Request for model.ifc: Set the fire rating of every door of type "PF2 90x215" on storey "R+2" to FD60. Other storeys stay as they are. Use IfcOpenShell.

First a look at what the model holds.

```python
import ifcopenshell
import ifcopenshell.util.element

model = ifcopenshell.open("model.ifc")
print(model.schema)
storey = next(s for s in model.by_type("IfcBuildingStorey") if s.Name == "R+2")
doors = [e for e in ifcopenshell.util.element.get_decomposition(storey) if e.is_a("IfcDoor")]
seen = {}
for e in doors:
    element_type = ifcopenshell.util.element.get_type(e)
    key = (element_type.Name if element_type != e and element_type else None, ifcopenshell.util.element.get_pset(e, "Pset_DoorCommon", "FireRating"))
    seen[key] = seen.get(key, 0) + 1
for (name, value), count in sorted(seen.items(), key=str):
    print(count, "x", name, "|", value)
```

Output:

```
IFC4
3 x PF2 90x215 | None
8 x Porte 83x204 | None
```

```python
import ifcopenshell
import ifcopenshell.api.pset
import ifcopenshell.util.element

model = ifcopenshell.open("model.ifc")

storey = next(s for s in model.by_type("IfcBuildingStorey") if s.Name == "R+2")
doors = [e for e in ifcopenshell.util.element.get_decomposition(storey) if e.is_a("IfcDoor")]

count = 0
for e in doors:
    element_type = ifcopenshell.util.element.get_type(e)
    if element_type in (None, e) or element_type.Name != "PF2 90x215":
        continue
    # add_pset returns the element's existing set when there is one.
    pset = ifcopenshell.api.pset.add_pset(model, product=e, name="Pset_DoorCommon")
    ifcopenshell.api.pset.edit_pset(model, pset=pset, properties={"FireRating": "FD60"})
    count += 1

print(count, "doors updated")

model.write("model_edited.ifc")
```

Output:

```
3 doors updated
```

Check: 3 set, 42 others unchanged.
